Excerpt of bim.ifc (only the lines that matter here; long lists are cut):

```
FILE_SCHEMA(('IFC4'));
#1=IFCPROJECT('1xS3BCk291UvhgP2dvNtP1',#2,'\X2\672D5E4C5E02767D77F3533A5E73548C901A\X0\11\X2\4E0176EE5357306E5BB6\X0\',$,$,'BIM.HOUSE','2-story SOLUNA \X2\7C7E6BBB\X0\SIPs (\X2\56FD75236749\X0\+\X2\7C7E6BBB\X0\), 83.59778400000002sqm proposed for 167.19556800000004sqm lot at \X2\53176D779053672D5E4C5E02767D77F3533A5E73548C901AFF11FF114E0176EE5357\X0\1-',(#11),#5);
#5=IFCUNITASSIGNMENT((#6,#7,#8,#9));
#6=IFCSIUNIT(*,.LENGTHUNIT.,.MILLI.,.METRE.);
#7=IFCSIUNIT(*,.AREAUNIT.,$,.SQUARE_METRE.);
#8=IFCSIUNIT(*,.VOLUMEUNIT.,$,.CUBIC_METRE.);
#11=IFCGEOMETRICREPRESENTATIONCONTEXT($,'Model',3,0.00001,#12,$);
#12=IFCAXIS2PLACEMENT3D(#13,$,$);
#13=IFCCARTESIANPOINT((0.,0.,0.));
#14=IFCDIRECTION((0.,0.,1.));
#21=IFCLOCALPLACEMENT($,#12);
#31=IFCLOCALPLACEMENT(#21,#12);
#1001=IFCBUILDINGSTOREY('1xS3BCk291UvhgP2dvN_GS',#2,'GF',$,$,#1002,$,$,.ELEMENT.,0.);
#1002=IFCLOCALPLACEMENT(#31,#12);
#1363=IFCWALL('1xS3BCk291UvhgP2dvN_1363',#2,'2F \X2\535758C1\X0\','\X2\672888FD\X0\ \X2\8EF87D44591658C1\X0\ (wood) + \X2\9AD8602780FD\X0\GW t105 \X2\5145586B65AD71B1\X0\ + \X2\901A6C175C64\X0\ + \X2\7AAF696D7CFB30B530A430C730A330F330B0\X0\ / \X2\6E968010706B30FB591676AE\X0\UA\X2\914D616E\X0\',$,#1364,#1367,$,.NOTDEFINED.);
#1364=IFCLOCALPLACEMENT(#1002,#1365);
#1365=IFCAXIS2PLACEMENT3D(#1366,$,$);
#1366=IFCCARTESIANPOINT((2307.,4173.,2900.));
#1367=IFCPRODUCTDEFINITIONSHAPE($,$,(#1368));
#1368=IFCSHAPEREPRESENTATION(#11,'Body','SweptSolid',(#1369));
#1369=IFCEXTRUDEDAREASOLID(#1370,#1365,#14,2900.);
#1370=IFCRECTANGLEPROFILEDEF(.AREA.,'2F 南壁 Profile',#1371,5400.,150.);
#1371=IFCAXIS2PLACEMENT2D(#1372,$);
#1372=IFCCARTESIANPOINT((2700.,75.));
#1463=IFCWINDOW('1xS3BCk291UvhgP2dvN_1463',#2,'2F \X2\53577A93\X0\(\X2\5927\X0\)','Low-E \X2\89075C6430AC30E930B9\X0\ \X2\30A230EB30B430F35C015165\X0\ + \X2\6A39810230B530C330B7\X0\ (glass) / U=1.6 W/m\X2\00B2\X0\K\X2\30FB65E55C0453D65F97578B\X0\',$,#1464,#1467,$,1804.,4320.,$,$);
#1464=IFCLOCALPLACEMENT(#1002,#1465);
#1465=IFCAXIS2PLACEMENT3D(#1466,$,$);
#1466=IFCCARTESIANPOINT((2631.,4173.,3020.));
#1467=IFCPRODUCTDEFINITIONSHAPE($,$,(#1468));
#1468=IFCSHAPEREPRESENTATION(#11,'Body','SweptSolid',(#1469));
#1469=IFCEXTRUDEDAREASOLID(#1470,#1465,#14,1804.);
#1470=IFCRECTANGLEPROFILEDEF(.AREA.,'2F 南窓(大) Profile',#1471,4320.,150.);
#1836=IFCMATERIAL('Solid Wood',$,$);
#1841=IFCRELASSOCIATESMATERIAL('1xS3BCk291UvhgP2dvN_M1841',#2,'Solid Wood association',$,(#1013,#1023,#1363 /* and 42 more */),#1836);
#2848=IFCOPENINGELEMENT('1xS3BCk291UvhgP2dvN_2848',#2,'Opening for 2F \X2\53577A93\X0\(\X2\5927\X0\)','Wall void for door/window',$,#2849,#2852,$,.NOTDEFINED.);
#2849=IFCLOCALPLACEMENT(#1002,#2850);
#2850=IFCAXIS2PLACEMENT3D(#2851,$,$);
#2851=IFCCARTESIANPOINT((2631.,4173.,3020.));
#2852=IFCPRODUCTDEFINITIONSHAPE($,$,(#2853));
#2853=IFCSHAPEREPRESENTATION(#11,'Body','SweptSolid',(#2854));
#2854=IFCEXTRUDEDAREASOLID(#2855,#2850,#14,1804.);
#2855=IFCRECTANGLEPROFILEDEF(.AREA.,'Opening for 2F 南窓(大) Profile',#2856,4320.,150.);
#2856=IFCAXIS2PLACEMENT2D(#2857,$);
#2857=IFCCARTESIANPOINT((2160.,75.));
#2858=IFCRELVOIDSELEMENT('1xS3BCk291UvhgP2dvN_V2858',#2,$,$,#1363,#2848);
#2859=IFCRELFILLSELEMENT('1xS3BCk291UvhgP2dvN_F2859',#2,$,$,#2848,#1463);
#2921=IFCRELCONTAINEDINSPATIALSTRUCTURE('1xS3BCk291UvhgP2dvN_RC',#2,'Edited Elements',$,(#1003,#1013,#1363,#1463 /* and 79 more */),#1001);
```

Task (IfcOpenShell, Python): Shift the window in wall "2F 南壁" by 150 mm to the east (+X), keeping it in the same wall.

```python
import ifcopenshell
import ifcopenshell.api.geometry
import ifcopenshell.util.placement
import ifcopenshell.util.unit

model = ifcopenshell.open("bim.ifc")
unit_scale = ifcopenshell.util.unit.calculate_unit_scale(model)

window = model.by_guid("1xS3BCk291UvhgP2dvN_1463")
opening = window.FillsVoids[0].RelatingOpeningElement
wall = opening.VoidsElements[0].RelatingBuildingElement

wall_matrix = ifcopenshell.util.placement.get_local_placement(wall.ObjectPlacement)
shift = wall_matrix[:3, 0] * 0.15 / unit_scale
before = ifcopenshell.util.placement.get_local_placement(window.ObjectPlacement)[:3, 3].copy()

# The window is not placed relative to its opening, so move both.
for product in (opening, window):
    matrix = ifcopenshell.util.placement.get_local_placement(product.ObjectPlacement)
    matrix[:3, 3] += shift
    ifcopenshell.api.geometry.edit_object_placement(model, product=product, matrix=matrix, is_si=False)

after = ifcopenshell.util.placement.get_local_placement(window.ObjectPlacement)[:3, 3]
print("window moved by", (after - before).round(3) + 0.0)

model.write("bim_rev.ifc")
```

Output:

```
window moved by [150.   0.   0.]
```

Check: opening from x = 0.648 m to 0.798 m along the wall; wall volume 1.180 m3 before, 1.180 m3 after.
